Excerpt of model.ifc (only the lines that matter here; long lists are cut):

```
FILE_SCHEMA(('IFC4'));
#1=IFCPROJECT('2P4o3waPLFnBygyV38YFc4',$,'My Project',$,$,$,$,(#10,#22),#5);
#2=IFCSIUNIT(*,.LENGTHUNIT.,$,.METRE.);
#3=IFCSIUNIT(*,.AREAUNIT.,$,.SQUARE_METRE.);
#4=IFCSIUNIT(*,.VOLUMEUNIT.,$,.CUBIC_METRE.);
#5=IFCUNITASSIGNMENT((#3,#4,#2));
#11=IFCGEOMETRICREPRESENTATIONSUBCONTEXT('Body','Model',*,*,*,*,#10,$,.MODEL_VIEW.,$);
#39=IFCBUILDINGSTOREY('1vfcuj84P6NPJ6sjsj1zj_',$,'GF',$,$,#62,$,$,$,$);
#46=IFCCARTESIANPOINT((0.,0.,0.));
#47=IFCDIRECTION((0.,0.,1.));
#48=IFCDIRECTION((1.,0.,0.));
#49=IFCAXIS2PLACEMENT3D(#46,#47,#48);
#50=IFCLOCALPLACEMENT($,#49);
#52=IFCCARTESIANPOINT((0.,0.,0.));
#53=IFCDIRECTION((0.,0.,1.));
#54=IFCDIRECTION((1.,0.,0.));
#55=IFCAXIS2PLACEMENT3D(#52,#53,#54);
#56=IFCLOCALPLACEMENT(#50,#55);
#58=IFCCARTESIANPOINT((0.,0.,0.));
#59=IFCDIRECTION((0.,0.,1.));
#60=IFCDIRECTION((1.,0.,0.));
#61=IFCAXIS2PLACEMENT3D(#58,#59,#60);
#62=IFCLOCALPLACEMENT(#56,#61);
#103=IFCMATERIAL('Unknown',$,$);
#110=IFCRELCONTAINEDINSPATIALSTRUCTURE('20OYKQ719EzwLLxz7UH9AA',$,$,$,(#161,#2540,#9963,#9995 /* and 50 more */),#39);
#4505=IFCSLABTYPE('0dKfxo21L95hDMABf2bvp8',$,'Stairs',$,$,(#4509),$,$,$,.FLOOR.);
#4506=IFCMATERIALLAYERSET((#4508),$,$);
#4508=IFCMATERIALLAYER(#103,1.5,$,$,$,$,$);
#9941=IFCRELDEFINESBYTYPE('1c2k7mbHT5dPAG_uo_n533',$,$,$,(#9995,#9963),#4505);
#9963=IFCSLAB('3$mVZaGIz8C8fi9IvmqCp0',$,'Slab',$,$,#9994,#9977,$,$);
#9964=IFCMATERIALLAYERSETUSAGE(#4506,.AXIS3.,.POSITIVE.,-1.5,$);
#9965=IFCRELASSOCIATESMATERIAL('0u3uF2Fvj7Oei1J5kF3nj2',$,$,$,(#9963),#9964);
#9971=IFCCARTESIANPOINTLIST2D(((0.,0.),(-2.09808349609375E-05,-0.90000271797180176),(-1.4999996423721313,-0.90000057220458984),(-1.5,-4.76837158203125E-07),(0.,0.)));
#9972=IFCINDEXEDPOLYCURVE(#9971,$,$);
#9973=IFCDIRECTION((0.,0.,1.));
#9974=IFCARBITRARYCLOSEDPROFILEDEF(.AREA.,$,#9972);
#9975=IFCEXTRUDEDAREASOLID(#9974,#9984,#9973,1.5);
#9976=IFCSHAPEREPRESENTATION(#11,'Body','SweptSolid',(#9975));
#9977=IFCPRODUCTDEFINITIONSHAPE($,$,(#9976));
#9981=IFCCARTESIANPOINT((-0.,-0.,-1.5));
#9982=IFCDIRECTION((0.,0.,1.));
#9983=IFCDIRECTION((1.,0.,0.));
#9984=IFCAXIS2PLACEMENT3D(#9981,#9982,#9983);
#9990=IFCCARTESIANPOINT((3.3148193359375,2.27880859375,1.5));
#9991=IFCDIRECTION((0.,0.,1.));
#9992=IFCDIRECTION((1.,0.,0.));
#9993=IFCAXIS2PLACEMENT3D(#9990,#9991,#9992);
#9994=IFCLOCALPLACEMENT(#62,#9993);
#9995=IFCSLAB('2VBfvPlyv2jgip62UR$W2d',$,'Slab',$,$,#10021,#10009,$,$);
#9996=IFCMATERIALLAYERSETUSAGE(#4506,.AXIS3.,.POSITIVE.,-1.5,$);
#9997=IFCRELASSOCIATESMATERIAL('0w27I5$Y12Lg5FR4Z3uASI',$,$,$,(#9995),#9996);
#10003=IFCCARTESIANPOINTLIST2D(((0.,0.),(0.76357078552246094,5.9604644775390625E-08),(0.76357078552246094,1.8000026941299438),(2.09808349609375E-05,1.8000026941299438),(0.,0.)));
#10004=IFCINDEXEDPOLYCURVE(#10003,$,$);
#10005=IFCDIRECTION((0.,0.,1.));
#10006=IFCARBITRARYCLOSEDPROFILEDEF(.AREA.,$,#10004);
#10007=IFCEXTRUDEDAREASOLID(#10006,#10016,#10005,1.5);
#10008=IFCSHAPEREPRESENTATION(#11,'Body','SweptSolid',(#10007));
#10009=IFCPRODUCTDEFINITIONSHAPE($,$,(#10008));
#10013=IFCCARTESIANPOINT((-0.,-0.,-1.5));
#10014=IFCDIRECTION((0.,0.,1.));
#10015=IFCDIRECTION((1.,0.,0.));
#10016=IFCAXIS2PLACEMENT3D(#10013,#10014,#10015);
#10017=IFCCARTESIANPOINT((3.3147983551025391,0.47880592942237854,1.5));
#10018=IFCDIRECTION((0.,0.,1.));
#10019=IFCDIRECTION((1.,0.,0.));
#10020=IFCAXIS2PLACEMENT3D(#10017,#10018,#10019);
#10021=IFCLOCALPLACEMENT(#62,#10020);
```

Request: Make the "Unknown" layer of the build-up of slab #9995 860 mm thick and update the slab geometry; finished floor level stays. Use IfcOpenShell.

```python
import ifcopenshell
import ifcopenshell.util.element
import ifcopenshell.util.representation

model = ifcopenshell.open("model.ifc")

layer_set = model.by_id(4506)
layer = next(l for l in layer_set.MaterialLayers if l.Material and l.Material.Name == "Unknown")
change = 0.86 - layer.LayerThickness
layer.LayerThickness += change

# The layer set is shared, so every slab that uses it gets the new thickness.
slabs = [e for e in ifcopenshell.util.element.get_elements_by_material(model, layer_set) if e.is_a("IfcSlab")]
for slab in sorted(slabs, key=lambda e: e.id()):
    body = ifcopenshell.util.representation.get_representation(slab, "Model", "Body")
    solid = body.Items[0]
    old_depth = solid.Depth
    solid.Depth += change
    # Extruded upwards: lower the start of the extrusion so the top stays.
    x, y, z = solid.Position.Location.Coordinates
    solid.Position.Location = model.createIfcCartesianPoint((x, y, z - change))
    print(slab.id(), f"{old_depth:g} -> {solid.Depth:g}")

# The layers are counted up from the underside, which has moved.
for usage in {ifcopenshell.util.element.get_material(slab) for slab in slabs}:
    usage.OffsetFromReferenceLine -= change

model.write("model_edited.ifc")
```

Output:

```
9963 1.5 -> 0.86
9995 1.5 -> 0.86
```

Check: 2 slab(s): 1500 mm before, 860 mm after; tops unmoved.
